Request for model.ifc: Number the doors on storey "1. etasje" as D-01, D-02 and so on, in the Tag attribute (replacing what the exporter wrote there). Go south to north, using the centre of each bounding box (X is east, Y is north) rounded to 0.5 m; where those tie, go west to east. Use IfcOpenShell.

First a look at what the model holds.

```python
import ifcopenshell
import ifcopenshell.util.element
import ifcopenshell.util.placement

model = ifcopenshell.open("model.ifc")
print(model.schema)
storey = next(s for s in model.by_type("IfcBuildingStorey") if s.Name == "1. etasje")
doors = [e for e in ifcopenshell.util.element.get_decomposition(storey) if e.is_a("IfcDoor")]
for e in sorted(doors, key=lambda e: e.id()):
    origin = ifcopenshell.util.placement.get_local_placement(e.ObjectPlacement)[:3, 3]
    print(e.id(), e.Tag, e.Name, origin.round(2) + 0.0, sep=" | ")
```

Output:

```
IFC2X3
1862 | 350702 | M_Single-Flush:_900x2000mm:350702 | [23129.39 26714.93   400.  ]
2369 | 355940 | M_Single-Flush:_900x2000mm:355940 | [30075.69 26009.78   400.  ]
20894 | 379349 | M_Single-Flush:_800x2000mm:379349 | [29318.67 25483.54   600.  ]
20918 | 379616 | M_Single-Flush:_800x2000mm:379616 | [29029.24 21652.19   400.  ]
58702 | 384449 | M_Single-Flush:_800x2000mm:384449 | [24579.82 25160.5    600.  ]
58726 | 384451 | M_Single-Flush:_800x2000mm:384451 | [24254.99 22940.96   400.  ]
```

```python
import ifcopenshell
import ifcopenshell.geom
import ifcopenshell.util.element
import ifcopenshell.util.shape

model = ifcopenshell.open("model.ifc")
settings = ifcopenshell.geom.settings()
settings.set("use-world-coords", True)


def centre(element):
    shape = ifcopenshell.geom.create_shape(settings, element)
    return ifcopenshell.util.shape.get_bbox_centroid(shape.geometry)


storey = next(s for s in model.by_type("IfcBuildingStorey") if s.Name == "1. etasje")
doors = [e for e in ifcopenshell.util.element.get_decomposition(storey) if e.is_a("IfcDoor")]

# Insertion points can sit at a corner or the storey origin, so sort by the geometry (in metres).
centres = {e: centre(e) for e in doors}
doors.sort(key=lambda e: (round(centres[e][1] / 0.5), centres[e][0]))

for i, e in enumerate(doors, start=1):
    number = f"D-{i:02d}"
    e.Tag = number
    print(e.id(), number)

model.write("model-out.ifc")
```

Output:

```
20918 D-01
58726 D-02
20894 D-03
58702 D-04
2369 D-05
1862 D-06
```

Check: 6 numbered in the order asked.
